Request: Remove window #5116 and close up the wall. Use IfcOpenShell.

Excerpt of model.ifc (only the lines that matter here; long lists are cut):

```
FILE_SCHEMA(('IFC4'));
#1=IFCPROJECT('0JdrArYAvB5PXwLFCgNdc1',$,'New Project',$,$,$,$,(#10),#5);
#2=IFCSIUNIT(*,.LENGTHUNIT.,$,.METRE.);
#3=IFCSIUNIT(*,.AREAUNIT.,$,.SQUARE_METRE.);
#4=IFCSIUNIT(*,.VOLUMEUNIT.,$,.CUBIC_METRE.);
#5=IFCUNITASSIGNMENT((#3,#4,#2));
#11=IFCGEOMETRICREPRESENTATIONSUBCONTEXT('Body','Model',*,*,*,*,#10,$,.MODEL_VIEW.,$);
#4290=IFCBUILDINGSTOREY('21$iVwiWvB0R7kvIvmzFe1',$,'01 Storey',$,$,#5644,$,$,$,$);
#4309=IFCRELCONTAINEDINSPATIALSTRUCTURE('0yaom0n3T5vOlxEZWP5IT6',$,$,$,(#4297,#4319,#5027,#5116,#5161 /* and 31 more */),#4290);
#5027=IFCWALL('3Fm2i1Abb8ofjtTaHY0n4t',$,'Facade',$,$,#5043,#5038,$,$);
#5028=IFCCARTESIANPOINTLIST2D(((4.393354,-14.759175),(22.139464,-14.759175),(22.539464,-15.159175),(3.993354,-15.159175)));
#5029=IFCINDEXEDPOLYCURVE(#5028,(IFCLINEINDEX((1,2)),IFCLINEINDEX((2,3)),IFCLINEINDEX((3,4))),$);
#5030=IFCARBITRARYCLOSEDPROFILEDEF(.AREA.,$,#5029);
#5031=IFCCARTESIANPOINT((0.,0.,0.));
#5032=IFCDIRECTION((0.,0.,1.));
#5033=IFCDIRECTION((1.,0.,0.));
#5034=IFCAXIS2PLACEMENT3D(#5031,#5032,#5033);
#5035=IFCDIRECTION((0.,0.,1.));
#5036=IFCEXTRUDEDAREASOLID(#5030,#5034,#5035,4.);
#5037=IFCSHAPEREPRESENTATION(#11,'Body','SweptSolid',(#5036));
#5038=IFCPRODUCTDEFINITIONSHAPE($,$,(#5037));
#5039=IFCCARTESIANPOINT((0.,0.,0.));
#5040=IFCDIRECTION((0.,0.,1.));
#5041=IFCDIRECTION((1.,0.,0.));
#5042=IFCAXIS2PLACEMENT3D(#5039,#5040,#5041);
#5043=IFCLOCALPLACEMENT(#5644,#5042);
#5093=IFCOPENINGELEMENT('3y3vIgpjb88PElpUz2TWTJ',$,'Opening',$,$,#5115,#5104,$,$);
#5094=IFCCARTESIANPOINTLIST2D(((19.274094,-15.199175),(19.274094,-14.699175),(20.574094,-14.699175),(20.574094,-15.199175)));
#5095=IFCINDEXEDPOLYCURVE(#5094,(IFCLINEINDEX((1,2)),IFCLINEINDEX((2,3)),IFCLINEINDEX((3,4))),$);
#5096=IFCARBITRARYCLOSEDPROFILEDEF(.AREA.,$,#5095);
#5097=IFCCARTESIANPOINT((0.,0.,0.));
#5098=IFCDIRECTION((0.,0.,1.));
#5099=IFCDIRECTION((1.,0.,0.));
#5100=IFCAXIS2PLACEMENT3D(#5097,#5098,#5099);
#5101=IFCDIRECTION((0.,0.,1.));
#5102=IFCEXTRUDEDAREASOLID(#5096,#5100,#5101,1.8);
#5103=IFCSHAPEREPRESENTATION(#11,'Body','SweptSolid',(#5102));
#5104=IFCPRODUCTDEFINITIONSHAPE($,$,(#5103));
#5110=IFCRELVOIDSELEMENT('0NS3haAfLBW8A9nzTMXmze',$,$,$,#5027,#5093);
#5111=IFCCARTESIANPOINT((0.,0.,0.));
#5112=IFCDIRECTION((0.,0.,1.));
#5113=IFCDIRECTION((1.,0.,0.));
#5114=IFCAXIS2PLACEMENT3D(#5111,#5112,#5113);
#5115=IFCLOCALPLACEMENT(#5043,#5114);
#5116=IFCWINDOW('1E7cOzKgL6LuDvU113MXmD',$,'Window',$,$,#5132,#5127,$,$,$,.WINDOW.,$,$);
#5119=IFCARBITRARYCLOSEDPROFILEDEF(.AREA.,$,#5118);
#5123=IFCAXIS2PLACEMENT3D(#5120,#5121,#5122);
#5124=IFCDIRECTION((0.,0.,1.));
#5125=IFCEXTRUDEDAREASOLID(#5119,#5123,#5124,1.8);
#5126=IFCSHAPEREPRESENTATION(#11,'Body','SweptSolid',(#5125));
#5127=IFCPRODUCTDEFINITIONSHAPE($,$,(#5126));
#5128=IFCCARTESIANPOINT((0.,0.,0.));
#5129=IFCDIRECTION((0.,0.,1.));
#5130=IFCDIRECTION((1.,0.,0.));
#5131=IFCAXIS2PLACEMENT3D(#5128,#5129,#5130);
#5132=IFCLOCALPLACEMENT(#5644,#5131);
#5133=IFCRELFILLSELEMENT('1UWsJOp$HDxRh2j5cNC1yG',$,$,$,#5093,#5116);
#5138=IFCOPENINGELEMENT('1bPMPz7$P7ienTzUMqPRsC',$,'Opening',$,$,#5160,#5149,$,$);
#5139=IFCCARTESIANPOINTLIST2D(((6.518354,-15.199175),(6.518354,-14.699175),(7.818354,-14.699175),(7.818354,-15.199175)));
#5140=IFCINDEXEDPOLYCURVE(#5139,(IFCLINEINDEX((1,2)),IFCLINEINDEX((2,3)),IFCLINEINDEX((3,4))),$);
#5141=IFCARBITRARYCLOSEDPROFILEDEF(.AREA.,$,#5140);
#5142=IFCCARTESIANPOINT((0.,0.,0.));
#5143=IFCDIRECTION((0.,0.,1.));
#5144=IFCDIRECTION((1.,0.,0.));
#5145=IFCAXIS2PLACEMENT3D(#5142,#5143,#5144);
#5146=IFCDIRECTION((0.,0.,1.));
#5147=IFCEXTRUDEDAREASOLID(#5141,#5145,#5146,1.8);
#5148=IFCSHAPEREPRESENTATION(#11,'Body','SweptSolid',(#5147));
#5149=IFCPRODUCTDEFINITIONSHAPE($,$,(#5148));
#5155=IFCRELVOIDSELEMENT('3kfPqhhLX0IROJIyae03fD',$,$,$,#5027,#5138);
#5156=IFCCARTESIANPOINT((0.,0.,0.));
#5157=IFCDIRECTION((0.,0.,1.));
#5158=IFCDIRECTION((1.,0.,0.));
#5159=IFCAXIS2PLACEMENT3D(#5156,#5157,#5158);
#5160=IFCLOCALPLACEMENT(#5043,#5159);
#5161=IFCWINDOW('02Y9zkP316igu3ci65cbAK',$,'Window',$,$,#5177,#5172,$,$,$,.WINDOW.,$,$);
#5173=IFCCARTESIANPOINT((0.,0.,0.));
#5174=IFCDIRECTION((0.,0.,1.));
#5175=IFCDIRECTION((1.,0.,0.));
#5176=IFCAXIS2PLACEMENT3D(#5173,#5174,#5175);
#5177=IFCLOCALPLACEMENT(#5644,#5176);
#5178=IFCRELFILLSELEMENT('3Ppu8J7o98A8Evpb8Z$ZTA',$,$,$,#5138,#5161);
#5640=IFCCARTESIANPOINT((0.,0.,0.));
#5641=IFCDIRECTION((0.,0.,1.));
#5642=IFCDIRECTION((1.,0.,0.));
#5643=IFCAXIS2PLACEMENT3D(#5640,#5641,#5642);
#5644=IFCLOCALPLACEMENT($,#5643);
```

```python
import ifcopenshell
import ifcopenshell.api.feature
import ifcopenshell.api.root
import ifcopenshell.geom
import ifcopenshell.util.shape

model = ifcopenshell.open("model.ifc")
settings = ifcopenshell.geom.settings()


def volume(element):
    """Net volume in cubic metres, openings subtracted."""
    shape = ifcopenshell.geom.create_shape(settings, element)
    return ifcopenshell.util.shape.get_volume(shape.geometry)


window = model.by_id(5116)
opening = window.FillsVoids[0].RelatingOpeningElement
wall = opening.VoidsElements[0].RelatingBuildingElement
before = volume(wall)

ifcopenshell.api.root.remove_product(model, product=window)
ifcopenshell.api.feature.remove_feature(model, feature=opening)

after = volume(wall)

print(f"wall volume {before:.3f} -> {after:.3f} m3")

model.write("model_updated.ifc")
```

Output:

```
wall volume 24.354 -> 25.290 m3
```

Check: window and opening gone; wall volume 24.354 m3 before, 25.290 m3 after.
